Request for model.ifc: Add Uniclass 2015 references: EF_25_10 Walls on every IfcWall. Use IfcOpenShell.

First a look at what the model holds.

```python
import ifcopenshell

model = ifcopenshell.open("model.ifc")
print(model.schema)
print("classifications:", [c.Name for c in model.by_type("IfcClassification")])
for ifc_class in ("IfcDoor", "IfcRoof", "IfcStair", "IfcWall", "IfcWindow"):
    print(ifc_class, len(model.by_type(ifc_class)))
```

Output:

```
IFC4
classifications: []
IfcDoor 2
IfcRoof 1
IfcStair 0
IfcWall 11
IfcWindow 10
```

```python
import ifcopenshell
import ifcopenshell.api.classification

model = ifcopenshell.open("model.ifc")

system = ifcopenshell.api.classification.add_classification(model, classification="Uniclass 2015")

codes = {
    "IfcWall": ("EF_25_10", "Walls"),
}
for ifc_class, (code, name) in codes.items():
    products = model.by_type(ifc_class)
    ifcopenshell.api.classification.add_reference(
        model, products=products, classification=system, identification=code, name=name
    )
    print(code, len(products))

model.write("model_updated.ifc")
```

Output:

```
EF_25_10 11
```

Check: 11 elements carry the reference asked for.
